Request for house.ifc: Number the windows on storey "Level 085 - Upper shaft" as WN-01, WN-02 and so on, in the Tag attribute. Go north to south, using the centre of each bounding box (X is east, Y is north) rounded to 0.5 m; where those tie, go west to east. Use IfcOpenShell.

First a look at what the model holds.

```python
import ifcopenshell
import ifcopenshell.util.element
import ifcopenshell.util.placement

model = ifcopenshell.open("house.ifc")
print(model.schema)
storey = next(s for s in model.by_type("IfcBuildingStorey") if s.Name == "Level 085 - Upper shaft")
windows = [e for e in ifcopenshell.util.element.get_decomposition(storey) if e.is_a("IfcWindow")]
for e in sorted(windows, key=lambda e: e.id()):
    origin = ifcopenshell.util.placement.get_local_placement(e.ObjectPlacement)[:3, 3]
    print(e.id(), e.Tag, e.Name, origin.round(2) + 0.0, sep=" | ")
```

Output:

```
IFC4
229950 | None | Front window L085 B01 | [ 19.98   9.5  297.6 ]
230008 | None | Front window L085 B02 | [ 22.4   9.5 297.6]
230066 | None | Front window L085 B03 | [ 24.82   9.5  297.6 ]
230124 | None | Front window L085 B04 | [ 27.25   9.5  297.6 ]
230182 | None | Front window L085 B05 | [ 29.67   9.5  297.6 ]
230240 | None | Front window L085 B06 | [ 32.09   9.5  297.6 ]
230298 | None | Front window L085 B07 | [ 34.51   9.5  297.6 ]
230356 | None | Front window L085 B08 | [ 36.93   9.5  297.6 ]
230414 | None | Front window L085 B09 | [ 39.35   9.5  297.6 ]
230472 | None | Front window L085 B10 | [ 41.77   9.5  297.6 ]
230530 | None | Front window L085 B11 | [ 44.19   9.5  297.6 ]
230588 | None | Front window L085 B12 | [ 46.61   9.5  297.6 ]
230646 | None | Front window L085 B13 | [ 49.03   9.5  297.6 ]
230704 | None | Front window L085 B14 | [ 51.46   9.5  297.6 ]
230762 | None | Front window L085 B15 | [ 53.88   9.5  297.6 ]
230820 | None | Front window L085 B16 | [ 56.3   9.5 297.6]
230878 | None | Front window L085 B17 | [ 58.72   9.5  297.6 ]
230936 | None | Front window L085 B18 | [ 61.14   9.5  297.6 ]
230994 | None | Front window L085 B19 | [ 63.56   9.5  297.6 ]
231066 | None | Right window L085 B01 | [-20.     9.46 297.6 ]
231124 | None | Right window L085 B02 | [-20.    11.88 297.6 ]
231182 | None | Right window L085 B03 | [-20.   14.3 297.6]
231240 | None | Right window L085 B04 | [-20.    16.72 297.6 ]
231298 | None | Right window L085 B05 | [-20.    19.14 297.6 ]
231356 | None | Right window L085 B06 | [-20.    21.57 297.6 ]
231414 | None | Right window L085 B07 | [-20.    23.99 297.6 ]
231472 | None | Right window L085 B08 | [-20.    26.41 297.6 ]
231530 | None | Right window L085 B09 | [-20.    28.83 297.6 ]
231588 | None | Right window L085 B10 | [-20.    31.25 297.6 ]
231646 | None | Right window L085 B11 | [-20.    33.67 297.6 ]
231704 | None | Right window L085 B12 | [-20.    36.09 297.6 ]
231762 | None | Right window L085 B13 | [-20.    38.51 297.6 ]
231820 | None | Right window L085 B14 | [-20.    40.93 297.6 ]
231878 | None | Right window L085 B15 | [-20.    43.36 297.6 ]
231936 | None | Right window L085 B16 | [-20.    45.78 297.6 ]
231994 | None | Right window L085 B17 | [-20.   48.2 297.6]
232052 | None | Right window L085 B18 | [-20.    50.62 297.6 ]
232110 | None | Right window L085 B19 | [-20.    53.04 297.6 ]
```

```python
import ifcopenshell
import ifcopenshell.geom
import ifcopenshell.util.element
import ifcopenshell.util.shape

model = ifcopenshell.open("house.ifc")
settings = ifcopenshell.geom.settings()
settings.set("use-world-coords", True)


def centre(element):
    shape = ifcopenshell.geom.create_shape(settings, element)
    return ifcopenshell.util.shape.get_bbox_centroid(shape.geometry)


storey = next(s for s in model.by_type("IfcBuildingStorey") if s.Name == "Level 085 - Upper shaft")
windows = [e for e in ifcopenshell.util.element.get_decomposition(storey) if e.is_a("IfcWindow")]

# Insertion points can sit at a corner or the storey origin, so sort by the geometry (in metres).
centres = {e: centre(e) for e in windows}
windows.sort(key=lambda e: (-round(centres[e][1] / 0.5), centres[e][0]))

for i, e in enumerate(windows, start=1):
    number = f"WN-{i:02d}"
    e.Tag = number
    print(e.id(), number)

model.write("house_rev.ifc")
```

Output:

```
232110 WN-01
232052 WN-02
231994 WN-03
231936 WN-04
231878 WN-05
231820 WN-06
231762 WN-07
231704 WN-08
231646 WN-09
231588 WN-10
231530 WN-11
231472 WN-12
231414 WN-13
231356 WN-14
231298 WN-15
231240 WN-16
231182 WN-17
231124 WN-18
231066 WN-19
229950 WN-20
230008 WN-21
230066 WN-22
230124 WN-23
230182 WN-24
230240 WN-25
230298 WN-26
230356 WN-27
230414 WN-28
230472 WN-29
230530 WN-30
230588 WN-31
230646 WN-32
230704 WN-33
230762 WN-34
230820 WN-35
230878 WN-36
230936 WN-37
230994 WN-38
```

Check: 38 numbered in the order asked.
